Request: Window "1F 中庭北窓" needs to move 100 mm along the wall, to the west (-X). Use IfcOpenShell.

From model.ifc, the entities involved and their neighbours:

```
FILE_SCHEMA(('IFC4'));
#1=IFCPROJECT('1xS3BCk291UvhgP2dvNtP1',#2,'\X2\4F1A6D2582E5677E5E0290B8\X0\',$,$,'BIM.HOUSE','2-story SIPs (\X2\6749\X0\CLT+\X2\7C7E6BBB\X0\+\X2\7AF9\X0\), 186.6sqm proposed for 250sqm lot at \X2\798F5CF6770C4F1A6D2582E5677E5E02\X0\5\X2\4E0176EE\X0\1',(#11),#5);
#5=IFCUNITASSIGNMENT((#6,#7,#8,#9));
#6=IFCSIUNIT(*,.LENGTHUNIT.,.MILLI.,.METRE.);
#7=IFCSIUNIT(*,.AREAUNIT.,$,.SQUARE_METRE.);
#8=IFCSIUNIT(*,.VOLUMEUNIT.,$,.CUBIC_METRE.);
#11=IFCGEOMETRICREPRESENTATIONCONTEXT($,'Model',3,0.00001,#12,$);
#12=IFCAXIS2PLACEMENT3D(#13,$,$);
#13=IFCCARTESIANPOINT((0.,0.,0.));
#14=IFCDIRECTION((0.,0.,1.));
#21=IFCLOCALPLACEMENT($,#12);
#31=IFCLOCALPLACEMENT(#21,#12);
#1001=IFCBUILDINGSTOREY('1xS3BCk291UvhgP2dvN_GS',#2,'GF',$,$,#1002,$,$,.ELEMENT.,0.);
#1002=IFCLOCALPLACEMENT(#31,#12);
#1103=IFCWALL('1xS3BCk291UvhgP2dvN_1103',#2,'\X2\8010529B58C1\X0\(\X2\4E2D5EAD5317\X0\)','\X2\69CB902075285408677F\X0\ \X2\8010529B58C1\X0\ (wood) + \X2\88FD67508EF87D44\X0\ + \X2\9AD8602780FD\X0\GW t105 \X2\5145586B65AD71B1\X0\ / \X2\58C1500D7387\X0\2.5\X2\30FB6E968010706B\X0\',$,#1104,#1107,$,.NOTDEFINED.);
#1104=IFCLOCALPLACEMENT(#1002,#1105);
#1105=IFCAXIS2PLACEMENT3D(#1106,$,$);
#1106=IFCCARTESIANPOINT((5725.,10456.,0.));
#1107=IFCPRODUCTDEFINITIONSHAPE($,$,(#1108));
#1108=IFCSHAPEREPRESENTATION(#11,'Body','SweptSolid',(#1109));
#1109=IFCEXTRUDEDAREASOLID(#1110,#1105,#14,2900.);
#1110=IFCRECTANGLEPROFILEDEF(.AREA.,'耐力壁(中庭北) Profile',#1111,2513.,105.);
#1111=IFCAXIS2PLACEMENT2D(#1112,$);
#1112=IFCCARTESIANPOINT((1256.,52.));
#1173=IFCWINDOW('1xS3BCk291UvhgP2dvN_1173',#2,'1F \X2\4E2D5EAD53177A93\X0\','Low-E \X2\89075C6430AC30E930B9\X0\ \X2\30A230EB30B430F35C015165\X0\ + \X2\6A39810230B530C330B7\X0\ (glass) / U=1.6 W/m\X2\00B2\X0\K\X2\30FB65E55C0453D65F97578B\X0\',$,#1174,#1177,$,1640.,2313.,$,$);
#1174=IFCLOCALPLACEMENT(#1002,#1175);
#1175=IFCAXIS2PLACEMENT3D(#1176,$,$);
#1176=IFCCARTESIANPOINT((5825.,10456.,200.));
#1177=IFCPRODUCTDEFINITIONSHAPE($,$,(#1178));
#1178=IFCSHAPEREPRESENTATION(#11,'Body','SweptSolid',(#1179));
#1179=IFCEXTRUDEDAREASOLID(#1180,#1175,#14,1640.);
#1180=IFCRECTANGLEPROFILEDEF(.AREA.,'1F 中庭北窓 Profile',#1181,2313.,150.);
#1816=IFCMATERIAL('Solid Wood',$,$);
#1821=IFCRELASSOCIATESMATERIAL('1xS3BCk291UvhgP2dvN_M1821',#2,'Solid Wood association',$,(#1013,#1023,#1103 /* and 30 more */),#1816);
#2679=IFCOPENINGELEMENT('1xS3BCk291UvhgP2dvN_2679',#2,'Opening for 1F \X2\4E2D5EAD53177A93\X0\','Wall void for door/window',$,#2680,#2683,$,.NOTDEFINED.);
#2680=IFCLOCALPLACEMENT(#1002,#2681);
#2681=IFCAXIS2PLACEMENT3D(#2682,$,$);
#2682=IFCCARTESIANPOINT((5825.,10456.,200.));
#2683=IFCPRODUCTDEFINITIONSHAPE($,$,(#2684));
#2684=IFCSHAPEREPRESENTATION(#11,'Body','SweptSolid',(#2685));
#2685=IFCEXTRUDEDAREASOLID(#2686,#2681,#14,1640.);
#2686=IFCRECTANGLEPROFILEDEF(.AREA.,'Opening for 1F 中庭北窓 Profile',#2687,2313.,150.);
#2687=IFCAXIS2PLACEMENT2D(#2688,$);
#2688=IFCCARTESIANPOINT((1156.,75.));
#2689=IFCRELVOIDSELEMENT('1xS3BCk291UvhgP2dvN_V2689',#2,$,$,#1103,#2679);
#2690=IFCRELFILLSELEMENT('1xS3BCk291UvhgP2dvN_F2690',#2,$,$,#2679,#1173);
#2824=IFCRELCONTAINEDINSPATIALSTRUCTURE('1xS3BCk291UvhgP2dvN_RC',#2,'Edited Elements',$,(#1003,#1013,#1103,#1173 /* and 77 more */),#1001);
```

```python
import ifcopenshell
import ifcopenshell.api.geometry
import ifcopenshell.util.placement

model = ifcopenshell.open("model.ifc")

window = model.by_guid("1xS3BCk291UvhgP2dvN_1173")
opening = window.FillsVoids[0].RelatingOpeningElement
wall = opening.VoidsElements[0].RelatingBuildingElement

wall_matrix = ifcopenshell.util.placement.get_local_placement(wall.ObjectPlacement)
shift = wall_matrix[:3, 0] * -100.0
before = ifcopenshell.util.placement.get_local_placement(window.ObjectPlacement)[:3, 3].copy()

# The window is not placed relative to its opening, so move both.
for product in (opening, window):
    matrix = ifcopenshell.util.placement.get_local_placement(product.ObjectPlacement)
    matrix[:3, 3] += shift
    ifcopenshell.api.geometry.edit_object_placement(model, product=product, matrix=matrix, is_si=False)

after = ifcopenshell.util.placement.get_local_placement(window.ObjectPlacement)[:3, 3]
print("window moved by", (after - before).round(3) + 0.0)

model.write("model_rev.ifc")
```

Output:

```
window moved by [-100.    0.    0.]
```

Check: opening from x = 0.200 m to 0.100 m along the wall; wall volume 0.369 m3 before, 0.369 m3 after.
